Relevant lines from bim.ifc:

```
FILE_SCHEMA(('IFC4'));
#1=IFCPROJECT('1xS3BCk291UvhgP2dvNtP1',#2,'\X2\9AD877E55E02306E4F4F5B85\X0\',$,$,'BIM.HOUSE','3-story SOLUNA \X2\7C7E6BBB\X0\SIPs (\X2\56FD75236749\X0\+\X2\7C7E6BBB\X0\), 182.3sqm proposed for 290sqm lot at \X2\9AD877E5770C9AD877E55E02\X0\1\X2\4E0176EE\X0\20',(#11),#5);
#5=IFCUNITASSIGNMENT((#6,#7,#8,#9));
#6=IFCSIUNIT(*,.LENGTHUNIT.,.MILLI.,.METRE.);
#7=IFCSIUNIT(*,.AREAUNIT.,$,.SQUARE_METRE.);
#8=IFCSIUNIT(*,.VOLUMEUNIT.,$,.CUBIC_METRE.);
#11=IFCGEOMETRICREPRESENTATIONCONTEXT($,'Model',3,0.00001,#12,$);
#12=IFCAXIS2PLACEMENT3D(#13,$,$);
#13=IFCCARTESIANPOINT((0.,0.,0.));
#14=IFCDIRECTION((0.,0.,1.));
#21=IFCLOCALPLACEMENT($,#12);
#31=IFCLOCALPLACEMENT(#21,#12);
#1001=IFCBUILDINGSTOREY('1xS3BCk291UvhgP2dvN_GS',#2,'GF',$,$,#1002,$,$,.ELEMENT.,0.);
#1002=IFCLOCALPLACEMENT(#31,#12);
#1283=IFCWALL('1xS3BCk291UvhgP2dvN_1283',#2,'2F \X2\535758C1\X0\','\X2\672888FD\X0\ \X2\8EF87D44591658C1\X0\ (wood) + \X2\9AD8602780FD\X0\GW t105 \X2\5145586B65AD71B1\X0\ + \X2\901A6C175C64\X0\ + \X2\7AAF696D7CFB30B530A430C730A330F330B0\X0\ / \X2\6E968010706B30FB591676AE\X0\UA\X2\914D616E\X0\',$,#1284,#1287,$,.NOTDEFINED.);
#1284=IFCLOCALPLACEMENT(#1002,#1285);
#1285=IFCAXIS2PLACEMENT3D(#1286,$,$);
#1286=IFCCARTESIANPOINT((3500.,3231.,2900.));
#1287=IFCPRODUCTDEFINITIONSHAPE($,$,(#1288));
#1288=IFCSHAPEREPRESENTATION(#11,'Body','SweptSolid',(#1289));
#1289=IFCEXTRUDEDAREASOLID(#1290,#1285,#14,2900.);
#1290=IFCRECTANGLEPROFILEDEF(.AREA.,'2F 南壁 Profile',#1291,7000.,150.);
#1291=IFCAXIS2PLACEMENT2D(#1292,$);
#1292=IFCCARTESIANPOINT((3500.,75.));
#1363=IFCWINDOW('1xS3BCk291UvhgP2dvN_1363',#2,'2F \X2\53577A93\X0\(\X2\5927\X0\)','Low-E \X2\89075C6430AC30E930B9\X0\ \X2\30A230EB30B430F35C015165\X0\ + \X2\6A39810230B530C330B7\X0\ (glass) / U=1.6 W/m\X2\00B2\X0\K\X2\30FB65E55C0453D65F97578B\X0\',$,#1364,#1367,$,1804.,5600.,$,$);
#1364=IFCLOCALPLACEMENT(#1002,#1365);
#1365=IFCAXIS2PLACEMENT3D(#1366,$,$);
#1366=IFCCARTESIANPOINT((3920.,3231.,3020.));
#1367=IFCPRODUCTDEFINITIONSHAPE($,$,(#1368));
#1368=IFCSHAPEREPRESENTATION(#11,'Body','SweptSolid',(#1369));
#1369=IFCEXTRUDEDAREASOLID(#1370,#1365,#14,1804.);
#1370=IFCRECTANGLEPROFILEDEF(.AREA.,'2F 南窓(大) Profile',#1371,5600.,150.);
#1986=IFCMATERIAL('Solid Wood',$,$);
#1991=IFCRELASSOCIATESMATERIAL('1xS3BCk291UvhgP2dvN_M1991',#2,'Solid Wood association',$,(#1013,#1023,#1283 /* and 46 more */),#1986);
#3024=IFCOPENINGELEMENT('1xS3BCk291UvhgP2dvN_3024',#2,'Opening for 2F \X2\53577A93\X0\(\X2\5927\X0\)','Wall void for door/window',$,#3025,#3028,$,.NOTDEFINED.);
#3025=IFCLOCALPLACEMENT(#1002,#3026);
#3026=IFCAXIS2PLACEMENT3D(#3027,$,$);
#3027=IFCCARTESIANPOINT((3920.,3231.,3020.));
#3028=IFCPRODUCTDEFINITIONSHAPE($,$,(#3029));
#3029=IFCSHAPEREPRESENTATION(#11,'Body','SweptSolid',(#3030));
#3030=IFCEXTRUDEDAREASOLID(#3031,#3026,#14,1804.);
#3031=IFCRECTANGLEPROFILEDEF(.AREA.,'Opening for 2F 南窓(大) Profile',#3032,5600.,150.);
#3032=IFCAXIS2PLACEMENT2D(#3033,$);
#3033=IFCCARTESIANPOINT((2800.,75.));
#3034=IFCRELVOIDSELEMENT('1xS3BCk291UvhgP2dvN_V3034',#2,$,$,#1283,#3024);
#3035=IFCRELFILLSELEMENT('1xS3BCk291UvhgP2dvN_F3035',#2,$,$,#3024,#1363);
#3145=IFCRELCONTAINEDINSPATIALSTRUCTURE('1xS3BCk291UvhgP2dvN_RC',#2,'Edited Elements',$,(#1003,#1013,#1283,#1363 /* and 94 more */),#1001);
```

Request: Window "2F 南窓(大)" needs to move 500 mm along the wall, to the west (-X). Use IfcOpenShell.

```python
import ifcopenshell
import ifcopenshell.api.geometry
import ifcopenshell.util.placement

model = ifcopenshell.open("bim.ifc")

window = model.by_guid("1xS3BCk291UvhgP2dvN_1363")
opening = window.FillsVoids[0].RelatingOpeningElement
wall = opening.VoidsElements[0].RelatingBuildingElement

wall_matrix = ifcopenshell.util.placement.get_local_placement(wall.ObjectPlacement)
shift = wall_matrix[:3, 0] * -500.0
before = ifcopenshell.util.placement.get_local_placement(window.ObjectPlacement)[:3, 3].copy()

# The window is not placed relative to its opening, so move both.
for product in (opening, window):
    matrix = ifcopenshell.util.placement.get_local_placement(product.ObjectPlacement)
    matrix[:3, 3] += shift
    ifcopenshell.api.geometry.edit_object_placement(model, product=product, matrix=matrix, is_si=False)

after = ifcopenshell.util.placement.get_local_placement(window.ObjectPlacement)[:3, 3]
print("window moved by", (after - before).round(3) + 0.0)

model.write("bim_edited.ifc")
```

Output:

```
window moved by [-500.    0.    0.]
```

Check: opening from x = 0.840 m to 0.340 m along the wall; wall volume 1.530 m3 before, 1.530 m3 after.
